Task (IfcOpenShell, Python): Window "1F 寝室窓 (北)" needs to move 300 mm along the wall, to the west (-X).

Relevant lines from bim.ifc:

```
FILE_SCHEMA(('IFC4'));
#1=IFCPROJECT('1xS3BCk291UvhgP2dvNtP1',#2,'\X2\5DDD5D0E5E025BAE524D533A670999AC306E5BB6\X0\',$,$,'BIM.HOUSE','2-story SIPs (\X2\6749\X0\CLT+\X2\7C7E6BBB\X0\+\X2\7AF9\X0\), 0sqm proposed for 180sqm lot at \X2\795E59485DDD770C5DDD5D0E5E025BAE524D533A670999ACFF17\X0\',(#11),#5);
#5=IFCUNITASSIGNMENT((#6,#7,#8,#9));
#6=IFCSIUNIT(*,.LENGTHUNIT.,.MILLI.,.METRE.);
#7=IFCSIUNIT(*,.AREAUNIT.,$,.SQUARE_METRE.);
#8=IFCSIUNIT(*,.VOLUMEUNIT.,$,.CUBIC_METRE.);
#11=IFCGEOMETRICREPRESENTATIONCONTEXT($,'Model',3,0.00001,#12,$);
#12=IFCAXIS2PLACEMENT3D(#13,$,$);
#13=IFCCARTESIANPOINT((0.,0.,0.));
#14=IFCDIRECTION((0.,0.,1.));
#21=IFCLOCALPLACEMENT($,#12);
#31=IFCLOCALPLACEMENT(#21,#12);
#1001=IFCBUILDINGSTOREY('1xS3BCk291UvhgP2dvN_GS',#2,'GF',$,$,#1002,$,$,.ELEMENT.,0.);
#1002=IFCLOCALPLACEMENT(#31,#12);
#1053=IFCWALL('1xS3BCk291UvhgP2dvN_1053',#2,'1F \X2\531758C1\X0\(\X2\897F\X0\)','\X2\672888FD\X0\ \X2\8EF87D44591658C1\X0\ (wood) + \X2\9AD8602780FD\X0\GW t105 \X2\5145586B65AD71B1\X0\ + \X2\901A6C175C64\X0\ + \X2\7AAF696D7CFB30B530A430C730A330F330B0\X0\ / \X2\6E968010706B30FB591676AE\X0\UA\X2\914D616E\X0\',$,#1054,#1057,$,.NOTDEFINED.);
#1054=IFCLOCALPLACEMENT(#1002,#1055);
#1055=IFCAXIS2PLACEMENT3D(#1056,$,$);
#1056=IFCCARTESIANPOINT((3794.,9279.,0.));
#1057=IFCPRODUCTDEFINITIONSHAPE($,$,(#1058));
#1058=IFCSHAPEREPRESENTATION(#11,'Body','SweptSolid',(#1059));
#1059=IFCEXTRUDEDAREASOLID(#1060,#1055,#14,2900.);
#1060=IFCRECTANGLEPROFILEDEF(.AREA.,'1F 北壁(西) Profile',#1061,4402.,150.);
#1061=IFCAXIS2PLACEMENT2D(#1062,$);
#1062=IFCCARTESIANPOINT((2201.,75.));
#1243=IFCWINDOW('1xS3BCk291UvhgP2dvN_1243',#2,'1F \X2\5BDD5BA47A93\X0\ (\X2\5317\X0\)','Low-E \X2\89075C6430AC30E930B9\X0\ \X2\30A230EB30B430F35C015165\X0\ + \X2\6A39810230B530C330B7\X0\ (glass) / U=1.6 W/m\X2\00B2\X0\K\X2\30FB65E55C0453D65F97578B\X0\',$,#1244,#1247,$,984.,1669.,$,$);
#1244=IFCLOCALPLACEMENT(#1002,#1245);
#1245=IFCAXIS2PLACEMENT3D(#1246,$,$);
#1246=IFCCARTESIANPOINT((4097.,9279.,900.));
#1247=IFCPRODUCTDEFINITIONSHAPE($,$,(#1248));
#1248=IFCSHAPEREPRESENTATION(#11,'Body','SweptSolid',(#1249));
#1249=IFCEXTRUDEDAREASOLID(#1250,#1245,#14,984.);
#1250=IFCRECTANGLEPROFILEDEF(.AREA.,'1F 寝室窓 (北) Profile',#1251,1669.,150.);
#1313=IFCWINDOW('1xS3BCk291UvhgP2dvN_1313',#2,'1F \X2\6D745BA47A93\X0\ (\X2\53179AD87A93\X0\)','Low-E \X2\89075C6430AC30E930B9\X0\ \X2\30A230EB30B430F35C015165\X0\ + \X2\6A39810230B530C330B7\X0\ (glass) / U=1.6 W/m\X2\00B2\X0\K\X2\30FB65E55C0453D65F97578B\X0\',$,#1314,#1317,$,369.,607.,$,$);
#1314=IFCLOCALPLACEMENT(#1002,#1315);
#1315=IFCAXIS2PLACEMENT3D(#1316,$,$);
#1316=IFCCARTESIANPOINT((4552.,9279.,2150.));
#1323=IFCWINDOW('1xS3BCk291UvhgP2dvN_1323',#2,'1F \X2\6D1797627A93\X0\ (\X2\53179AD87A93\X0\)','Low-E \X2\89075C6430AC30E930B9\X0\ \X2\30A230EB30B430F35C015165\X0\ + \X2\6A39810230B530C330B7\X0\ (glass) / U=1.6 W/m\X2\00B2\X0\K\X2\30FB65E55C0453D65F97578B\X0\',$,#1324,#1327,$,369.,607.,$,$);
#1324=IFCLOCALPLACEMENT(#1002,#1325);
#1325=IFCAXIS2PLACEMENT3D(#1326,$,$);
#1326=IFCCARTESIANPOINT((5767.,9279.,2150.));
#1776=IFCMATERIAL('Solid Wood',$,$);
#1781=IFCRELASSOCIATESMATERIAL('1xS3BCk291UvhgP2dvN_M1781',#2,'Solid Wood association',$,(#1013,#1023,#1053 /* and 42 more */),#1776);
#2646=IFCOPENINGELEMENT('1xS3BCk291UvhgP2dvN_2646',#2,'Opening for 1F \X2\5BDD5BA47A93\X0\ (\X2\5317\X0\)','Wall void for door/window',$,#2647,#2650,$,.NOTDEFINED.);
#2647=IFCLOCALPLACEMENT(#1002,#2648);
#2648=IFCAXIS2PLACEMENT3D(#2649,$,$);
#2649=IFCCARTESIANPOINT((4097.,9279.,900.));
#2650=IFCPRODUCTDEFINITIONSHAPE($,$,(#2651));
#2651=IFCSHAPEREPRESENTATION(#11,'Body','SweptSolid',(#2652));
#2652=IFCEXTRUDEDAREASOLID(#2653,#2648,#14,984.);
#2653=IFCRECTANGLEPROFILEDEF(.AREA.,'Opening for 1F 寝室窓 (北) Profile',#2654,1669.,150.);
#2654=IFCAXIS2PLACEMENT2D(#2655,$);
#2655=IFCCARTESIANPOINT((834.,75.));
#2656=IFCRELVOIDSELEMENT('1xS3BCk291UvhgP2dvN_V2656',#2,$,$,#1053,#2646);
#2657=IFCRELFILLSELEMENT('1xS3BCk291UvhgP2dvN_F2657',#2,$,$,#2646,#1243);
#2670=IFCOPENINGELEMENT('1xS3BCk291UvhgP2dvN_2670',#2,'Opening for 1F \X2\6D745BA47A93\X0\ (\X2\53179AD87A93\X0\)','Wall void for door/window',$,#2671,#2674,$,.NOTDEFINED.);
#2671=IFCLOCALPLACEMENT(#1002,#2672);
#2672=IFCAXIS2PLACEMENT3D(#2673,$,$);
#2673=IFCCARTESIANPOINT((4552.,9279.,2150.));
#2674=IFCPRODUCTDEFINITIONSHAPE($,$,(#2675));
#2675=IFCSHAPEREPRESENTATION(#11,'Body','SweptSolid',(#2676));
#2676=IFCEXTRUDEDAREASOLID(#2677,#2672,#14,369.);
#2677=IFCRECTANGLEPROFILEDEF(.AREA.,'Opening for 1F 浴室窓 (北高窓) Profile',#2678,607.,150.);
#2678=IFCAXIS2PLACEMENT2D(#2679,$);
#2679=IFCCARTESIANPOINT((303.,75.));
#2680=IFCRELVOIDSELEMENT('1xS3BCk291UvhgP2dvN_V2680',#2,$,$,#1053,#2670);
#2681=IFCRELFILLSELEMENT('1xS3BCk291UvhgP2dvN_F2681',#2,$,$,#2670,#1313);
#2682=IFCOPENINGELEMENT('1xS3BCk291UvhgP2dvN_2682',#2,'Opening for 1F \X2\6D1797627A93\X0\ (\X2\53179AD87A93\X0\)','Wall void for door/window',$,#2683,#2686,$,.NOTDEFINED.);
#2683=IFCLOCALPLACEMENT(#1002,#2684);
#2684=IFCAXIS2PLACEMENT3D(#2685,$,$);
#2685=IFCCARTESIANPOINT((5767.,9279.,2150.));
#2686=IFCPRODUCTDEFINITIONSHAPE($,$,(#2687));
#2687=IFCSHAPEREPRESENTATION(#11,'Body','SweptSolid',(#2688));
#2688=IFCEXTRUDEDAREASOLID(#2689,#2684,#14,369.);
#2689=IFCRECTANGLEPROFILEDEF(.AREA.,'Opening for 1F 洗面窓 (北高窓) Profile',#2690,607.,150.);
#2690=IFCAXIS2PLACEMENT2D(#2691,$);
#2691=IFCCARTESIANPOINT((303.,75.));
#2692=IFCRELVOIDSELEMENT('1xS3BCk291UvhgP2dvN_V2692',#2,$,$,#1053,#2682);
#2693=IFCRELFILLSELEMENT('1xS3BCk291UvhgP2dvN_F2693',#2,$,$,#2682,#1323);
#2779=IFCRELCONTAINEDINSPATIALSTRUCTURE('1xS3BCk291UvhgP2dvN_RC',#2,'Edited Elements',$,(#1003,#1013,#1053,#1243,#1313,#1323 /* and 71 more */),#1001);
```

```python
import ifcopenshell
import ifcopenshell.api.geometry
import ifcopenshell.util.placement

model = ifcopenshell.open("bim.ifc")

window = model.by_guid("1xS3BCk291UvhgP2dvN_1243")
opening = window.FillsVoids[0].RelatingOpeningElement
wall = opening.VoidsElements[0].RelatingBuildingElement

wall_matrix = ifcopenshell.util.placement.get_local_placement(wall.ObjectPlacement)
shift = wall_matrix[:3, 0] * -300.0
before = ifcopenshell.util.placement.get_local_placement(window.ObjectPlacement)[:3, 3].copy()

# The window is not placed relative to its opening, so move both.
for product in (opening, window):
    matrix = ifcopenshell.util.placement.get_local_placement(product.ObjectPlacement)
    matrix[:3, 3] += shift
    ifcopenshell.api.geometry.edit_object_placement(model, product=product, matrix=matrix, is_si=False)

after = ifcopenshell.util.placement.get_local_placement(window.ObjectPlacement)[:3, 3]
print("window moved by", (after - before).round(3) + 0.0)

model.write("bim_updated.ifc")
```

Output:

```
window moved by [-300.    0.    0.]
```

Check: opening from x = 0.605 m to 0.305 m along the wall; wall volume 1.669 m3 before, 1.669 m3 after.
